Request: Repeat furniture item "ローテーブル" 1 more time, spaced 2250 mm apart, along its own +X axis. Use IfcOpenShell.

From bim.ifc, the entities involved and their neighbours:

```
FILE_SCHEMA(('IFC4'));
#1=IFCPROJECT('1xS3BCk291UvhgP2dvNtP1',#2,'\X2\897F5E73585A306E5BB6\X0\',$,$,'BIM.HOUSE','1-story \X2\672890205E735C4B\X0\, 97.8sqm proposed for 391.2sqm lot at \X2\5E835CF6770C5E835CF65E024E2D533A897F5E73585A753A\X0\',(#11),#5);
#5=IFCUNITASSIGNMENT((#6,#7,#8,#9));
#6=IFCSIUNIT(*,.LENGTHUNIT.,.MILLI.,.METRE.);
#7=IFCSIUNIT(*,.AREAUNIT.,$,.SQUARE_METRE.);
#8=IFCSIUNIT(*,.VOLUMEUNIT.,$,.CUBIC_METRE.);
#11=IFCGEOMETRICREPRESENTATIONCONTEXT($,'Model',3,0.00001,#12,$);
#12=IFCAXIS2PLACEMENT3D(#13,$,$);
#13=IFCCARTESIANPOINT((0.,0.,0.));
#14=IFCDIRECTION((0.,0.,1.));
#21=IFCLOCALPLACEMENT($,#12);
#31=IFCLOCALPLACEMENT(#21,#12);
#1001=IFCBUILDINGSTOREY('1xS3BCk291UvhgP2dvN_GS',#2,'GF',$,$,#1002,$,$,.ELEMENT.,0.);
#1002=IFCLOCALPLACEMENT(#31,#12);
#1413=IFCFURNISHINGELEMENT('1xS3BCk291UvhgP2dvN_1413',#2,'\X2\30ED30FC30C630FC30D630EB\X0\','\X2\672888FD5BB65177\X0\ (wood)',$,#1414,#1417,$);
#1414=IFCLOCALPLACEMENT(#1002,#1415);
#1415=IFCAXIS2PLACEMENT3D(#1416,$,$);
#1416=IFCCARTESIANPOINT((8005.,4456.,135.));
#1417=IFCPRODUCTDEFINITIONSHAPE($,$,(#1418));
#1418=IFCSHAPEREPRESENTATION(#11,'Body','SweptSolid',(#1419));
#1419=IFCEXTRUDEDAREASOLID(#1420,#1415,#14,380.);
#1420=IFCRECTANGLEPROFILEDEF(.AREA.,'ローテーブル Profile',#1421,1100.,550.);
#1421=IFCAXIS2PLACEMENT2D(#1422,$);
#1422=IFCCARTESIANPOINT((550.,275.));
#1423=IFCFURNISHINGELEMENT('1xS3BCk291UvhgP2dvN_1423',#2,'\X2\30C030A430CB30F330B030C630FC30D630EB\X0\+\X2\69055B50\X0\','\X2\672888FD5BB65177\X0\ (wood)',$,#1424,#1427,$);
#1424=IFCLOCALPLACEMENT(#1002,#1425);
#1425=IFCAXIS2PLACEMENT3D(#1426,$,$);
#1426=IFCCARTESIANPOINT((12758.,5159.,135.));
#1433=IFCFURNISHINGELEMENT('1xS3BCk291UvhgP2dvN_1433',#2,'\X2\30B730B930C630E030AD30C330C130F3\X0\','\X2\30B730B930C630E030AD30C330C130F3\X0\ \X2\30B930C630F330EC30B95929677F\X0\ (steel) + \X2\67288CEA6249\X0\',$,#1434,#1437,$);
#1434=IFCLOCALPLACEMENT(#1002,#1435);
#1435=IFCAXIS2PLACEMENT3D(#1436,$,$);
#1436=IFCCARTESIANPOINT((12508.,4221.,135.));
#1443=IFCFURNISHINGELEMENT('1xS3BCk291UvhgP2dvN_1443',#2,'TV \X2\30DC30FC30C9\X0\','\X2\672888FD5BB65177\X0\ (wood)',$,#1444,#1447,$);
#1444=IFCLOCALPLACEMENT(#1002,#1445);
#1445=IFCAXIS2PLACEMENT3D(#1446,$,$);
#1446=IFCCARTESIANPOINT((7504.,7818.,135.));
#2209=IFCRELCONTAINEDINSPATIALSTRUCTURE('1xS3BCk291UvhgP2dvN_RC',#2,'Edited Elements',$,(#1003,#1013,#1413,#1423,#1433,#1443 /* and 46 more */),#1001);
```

```python
import ifcopenshell
import ifcopenshell.api.geometry
import ifcopenshell.api.root
import ifcopenshell.util.element
import ifcopenshell.util.placement
import ifcopenshell.util.unit

model = ifcopenshell.open("bim.ifc")
unit_scale = ifcopenshell.util.unit.calculate_unit_scale(model)


def reuse_history(source, copy):
    """copy_class also copies each property set's owner history, people and application; keep the originals."""
    for rel in copy.IsDefinedBy:
        if rel.is_a("IfcRelDefinesByProperties") and (history := rel.RelatingPropertyDefinition.OwnerHistory):
            rel.RelatingPropertyDefinition.OwnerHistory = source.OwnerHistory
            ifcopenshell.util.element.remove_deep2(model, history)


source = model.by_guid("1xS3BCk291UvhgP2dvN_1413")
base = ifcopenshell.util.placement.get_local_placement(source.ObjectPlacement)
step = base[:3, 0] * 2.25 / unit_scale

for i in range(1, 2):
    copy = ifcopenshell.api.root.copy_class(model, product=source)
    copy.Representation = ifcopenshell.util.element.copy_deep(
        model, source.Representation, exclude=["IfcGeometricRepresentationContext", "IfcRepresentationMap"]
    )
    reuse_history(source, copy)
    matrix = base.copy()
    matrix[:3, 3] += i * step
    print("added at", matrix[:3, 3].round(3) + 0.0)
    ifcopenshell.api.geometry.edit_object_placement(model, product=copy, matrix=matrix, is_si=False)

model.write("bim-out.ifc")
```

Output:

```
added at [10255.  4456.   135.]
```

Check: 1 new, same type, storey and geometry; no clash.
